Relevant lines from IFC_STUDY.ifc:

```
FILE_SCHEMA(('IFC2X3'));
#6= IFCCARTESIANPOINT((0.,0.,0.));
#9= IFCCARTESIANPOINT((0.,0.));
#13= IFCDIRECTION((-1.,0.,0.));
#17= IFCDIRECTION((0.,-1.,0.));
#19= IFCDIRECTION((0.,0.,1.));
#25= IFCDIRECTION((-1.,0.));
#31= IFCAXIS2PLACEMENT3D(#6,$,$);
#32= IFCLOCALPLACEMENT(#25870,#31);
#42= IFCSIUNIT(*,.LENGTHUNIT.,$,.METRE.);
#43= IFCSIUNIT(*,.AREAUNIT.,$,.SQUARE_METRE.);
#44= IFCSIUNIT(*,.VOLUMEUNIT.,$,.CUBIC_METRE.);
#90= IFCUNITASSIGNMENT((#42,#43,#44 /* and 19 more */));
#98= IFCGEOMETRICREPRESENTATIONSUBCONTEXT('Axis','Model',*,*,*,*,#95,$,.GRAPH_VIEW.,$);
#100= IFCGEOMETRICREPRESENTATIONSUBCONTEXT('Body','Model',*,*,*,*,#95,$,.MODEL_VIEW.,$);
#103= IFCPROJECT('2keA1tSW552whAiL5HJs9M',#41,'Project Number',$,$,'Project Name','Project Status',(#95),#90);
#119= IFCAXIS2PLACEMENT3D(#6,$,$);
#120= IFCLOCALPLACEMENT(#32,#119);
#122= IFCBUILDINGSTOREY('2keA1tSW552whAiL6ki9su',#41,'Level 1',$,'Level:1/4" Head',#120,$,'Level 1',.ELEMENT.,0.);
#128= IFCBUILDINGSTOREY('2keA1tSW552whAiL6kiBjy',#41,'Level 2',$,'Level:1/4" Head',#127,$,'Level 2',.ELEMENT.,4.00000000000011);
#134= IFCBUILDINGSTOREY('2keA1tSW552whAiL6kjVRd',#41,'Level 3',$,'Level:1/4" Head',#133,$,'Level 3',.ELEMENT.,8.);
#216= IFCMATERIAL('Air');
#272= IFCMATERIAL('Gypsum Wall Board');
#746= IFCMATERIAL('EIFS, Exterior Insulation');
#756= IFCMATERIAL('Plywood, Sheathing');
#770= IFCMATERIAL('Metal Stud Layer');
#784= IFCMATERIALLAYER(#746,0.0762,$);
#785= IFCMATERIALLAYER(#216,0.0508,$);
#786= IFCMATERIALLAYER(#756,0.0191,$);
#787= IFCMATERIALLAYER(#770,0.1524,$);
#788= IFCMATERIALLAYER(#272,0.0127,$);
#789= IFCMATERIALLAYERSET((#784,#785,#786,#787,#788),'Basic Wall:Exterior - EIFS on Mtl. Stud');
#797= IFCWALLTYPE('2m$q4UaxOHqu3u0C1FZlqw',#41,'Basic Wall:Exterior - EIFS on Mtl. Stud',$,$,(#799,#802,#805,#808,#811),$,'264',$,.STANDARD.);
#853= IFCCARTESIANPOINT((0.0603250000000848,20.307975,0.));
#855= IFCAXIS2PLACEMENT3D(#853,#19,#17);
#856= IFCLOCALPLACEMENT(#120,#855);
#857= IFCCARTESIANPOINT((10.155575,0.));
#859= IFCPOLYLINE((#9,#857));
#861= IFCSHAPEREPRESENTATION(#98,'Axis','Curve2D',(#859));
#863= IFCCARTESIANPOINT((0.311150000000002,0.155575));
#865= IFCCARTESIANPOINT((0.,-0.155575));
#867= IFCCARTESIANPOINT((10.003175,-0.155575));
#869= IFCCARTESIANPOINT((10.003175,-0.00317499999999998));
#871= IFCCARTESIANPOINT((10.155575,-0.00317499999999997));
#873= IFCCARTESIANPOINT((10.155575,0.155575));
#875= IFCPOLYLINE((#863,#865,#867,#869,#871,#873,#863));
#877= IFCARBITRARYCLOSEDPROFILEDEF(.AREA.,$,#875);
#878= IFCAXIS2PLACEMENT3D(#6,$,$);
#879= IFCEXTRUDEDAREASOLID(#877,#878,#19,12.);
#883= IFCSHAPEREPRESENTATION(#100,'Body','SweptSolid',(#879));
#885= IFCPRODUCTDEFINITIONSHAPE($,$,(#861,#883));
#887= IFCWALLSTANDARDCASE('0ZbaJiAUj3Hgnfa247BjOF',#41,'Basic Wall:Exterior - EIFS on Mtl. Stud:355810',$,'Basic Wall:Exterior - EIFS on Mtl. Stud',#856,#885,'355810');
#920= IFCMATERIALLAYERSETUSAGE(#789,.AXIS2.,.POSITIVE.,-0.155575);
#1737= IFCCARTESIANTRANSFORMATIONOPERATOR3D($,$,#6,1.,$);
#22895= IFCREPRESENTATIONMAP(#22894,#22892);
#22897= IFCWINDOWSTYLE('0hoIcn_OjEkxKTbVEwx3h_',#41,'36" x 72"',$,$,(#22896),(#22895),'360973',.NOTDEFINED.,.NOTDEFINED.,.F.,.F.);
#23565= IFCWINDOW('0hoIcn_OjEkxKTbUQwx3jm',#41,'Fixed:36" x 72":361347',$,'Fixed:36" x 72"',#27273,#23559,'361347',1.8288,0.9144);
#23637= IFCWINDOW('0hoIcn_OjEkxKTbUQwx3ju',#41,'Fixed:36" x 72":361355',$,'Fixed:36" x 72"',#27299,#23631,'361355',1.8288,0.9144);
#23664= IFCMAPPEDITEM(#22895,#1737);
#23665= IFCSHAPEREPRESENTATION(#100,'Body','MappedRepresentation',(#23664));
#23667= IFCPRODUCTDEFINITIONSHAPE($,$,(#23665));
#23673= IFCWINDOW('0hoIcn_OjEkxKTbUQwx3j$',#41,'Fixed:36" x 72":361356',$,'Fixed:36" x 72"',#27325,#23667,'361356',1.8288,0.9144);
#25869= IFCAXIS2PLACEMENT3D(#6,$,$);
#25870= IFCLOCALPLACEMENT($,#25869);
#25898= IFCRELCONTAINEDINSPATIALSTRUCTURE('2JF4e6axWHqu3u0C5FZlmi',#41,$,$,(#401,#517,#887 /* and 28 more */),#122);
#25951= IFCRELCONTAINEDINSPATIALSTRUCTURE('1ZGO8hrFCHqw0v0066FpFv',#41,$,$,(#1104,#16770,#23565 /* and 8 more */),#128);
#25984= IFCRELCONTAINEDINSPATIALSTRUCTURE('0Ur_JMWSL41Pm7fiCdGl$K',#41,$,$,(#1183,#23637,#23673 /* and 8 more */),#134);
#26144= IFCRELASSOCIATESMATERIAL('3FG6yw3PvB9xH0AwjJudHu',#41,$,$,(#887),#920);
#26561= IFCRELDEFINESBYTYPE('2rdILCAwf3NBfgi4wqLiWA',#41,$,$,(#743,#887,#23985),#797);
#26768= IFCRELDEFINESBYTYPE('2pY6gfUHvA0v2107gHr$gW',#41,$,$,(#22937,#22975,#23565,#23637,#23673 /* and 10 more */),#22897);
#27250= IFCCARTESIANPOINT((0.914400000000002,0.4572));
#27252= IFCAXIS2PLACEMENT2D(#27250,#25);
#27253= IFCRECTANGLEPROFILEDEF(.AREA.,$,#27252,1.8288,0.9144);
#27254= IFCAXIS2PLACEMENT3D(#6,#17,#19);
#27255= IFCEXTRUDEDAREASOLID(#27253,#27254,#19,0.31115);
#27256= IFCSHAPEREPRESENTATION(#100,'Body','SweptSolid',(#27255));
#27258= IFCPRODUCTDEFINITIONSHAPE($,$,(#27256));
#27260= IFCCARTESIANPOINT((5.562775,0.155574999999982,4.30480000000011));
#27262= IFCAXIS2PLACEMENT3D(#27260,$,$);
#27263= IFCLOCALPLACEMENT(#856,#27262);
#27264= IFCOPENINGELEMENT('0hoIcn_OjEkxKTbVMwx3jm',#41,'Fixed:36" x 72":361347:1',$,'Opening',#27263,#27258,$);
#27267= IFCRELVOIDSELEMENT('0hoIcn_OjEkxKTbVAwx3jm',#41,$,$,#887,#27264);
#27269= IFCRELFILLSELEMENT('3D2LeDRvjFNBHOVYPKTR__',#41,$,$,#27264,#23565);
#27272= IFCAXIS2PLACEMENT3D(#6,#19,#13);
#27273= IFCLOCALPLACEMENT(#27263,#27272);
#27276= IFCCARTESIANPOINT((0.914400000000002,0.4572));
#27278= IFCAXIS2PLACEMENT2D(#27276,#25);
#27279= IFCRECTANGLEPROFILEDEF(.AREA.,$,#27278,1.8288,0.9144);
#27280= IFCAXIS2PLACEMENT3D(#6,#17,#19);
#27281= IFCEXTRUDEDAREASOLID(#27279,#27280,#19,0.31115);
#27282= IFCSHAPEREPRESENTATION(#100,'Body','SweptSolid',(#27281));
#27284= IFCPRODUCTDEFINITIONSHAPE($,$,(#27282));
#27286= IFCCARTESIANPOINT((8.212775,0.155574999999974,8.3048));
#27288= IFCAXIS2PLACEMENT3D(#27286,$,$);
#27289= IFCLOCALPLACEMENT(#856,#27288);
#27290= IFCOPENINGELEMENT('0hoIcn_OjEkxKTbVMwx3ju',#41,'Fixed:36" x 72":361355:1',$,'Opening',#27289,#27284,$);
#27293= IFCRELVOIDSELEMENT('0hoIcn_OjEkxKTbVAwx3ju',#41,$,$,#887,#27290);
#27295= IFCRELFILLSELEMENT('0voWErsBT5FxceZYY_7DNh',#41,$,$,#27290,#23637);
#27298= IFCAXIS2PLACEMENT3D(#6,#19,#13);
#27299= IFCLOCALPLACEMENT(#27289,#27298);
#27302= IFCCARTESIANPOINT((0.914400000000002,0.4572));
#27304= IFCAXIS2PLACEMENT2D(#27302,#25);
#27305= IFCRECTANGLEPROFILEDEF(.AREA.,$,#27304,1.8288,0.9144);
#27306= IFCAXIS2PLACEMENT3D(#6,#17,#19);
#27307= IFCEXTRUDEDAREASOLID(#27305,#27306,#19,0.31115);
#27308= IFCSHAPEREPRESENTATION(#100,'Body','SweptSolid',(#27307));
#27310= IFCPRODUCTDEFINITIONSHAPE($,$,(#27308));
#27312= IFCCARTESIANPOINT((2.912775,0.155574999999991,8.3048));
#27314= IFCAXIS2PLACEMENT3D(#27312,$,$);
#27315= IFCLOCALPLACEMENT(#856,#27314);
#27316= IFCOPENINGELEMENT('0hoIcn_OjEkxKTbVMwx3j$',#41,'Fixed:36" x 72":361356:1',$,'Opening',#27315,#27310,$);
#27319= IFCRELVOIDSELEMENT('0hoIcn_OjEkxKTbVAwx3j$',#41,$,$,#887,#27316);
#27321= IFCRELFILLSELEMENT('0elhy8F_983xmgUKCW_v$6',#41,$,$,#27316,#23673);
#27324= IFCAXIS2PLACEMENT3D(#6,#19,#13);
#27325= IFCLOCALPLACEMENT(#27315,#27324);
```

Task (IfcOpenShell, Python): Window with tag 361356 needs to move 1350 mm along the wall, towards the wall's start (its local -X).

```python
import ifcopenshell
import ifcopenshell.api.geometry
import ifcopenshell.util.placement
import ifcopenshell.util.unit

model = ifcopenshell.open("IFC_STUDY.ifc")
unit_scale = ifcopenshell.util.unit.calculate_unit_scale(model)

window = model.by_id(23673)
opening = window.FillsVoids[0].RelatingOpeningElement
wall = opening.VoidsElements[0].RelatingBuildingElement

wall_matrix = ifcopenshell.util.placement.get_local_placement(wall.ObjectPlacement)
shift = wall_matrix[:3, 0] * -1.35 / unit_scale
before = ifcopenshell.util.placement.get_local_placement(window.ObjectPlacement)[:3, 3].copy()

# The window is placed relative to its opening, so it follows when the opening moves.
matrix = ifcopenshell.util.placement.get_local_placement(opening.ObjectPlacement)
matrix[:3, 3] += shift
ifcopenshell.api.geometry.edit_object_placement(
    model, product=opening, matrix=matrix, is_si=False, should_transform_children=True
)

after = ifcopenshell.util.placement.get_local_placement(window.ObjectPlacement)[:3, 3]
print("window moved by", (after - before).round(3) + 0.0)

model.write("IFC_STUDY_rev.ifc")
```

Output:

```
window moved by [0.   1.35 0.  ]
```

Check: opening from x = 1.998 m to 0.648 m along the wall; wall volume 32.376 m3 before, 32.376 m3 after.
